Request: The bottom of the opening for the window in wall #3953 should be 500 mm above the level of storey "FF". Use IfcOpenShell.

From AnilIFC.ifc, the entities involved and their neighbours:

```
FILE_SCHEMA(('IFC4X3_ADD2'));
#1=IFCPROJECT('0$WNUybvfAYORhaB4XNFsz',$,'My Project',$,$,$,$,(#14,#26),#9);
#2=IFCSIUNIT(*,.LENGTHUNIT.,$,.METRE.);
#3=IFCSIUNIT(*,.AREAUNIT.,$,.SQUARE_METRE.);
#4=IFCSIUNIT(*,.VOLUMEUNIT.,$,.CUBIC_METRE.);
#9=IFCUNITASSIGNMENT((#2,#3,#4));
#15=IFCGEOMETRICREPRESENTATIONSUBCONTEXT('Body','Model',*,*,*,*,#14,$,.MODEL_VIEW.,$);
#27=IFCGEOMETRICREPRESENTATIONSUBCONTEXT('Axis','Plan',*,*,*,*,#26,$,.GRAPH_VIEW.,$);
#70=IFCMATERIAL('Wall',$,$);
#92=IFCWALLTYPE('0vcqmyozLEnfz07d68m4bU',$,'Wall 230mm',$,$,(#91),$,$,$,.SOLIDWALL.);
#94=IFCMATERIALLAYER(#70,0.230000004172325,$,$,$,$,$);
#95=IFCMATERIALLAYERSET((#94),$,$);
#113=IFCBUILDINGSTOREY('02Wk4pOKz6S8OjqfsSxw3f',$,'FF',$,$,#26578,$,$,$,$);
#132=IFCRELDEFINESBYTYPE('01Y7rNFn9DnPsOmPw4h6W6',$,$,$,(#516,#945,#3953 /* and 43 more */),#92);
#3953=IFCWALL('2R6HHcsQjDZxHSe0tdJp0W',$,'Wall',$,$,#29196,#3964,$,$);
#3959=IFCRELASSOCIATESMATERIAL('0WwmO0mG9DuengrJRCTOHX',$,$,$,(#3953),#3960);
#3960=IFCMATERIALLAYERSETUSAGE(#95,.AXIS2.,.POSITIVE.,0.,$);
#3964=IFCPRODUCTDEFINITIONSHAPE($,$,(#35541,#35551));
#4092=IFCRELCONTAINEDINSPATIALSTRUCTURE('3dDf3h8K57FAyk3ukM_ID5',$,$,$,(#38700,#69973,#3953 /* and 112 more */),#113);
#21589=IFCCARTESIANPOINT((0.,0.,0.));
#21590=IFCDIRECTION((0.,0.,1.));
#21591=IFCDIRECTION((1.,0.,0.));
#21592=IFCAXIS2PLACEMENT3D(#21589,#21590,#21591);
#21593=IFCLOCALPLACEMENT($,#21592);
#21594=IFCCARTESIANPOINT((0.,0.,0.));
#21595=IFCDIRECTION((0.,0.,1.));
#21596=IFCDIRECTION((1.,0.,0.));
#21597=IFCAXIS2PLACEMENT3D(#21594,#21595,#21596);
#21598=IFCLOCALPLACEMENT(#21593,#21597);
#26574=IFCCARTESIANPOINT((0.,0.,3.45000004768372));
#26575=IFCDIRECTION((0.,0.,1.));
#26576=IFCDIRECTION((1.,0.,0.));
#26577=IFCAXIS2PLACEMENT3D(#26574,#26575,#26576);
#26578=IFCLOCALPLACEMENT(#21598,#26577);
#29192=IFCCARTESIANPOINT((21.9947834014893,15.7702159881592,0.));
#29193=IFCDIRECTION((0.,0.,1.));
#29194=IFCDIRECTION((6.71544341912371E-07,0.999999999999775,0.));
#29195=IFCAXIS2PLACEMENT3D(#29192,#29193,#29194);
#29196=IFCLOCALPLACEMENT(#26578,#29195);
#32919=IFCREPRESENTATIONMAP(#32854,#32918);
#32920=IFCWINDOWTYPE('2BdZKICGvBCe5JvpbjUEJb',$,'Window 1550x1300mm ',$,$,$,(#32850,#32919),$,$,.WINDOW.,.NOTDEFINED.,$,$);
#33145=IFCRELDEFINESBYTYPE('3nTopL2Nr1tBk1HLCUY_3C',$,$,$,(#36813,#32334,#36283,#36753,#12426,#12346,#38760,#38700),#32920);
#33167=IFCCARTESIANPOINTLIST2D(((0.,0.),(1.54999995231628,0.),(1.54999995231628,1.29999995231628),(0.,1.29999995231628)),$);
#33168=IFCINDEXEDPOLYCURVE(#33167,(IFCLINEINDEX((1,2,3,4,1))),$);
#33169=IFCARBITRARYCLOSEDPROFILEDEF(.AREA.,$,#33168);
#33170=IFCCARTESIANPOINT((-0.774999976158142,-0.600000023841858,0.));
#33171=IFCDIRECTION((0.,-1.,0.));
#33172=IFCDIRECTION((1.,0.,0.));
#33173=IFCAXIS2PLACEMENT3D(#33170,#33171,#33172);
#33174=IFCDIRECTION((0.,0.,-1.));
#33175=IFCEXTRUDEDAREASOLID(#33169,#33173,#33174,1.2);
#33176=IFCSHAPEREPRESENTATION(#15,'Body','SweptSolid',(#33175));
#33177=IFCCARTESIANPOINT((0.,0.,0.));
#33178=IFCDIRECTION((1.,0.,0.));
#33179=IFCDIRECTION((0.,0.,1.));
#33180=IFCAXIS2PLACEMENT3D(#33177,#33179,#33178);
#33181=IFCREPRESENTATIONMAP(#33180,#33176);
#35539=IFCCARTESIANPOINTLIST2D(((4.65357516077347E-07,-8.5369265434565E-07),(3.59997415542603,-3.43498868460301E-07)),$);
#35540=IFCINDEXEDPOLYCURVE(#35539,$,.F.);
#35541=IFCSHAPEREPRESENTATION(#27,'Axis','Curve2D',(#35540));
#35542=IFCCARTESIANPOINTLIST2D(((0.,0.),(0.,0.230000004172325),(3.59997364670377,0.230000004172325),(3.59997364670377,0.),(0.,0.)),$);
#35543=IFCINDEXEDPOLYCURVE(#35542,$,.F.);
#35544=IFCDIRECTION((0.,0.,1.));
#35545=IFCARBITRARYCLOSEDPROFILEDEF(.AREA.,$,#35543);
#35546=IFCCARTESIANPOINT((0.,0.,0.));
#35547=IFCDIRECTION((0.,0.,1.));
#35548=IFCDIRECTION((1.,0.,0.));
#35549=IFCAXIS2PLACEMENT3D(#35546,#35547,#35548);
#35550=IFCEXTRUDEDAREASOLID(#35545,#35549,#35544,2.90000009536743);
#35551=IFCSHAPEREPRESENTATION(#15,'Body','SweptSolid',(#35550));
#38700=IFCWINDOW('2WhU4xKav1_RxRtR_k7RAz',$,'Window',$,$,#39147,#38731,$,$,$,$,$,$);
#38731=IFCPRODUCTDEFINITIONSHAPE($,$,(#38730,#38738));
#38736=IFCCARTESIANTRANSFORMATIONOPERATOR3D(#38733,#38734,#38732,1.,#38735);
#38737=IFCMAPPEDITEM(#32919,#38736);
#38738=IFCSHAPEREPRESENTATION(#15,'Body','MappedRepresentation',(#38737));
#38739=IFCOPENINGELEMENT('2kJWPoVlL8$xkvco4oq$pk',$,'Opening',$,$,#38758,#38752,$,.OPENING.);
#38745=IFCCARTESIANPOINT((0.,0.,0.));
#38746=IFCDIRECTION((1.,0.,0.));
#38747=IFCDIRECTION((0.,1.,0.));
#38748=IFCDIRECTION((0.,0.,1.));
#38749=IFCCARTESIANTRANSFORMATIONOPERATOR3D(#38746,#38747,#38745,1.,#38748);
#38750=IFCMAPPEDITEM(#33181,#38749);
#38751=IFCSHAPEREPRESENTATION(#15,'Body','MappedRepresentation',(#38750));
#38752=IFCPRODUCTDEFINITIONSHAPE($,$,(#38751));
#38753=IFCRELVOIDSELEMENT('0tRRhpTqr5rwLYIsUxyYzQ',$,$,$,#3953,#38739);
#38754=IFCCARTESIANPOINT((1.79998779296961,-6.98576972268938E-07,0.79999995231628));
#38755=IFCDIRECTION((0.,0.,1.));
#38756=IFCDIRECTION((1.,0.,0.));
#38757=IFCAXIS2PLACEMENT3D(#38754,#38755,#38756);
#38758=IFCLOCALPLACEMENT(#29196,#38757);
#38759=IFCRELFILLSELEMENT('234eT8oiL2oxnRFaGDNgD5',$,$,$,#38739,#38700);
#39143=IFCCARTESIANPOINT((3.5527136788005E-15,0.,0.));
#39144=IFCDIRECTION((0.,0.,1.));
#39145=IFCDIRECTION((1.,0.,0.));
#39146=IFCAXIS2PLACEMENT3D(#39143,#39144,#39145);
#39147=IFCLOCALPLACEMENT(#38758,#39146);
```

```python
import numpy as np
import ifcopenshell
import ifcopenshell.api.geometry
import ifcopenshell.geom
import ifcopenshell.util.element
import ifcopenshell.util.placement
import ifcopenshell.util.shape
import ifcopenshell.util.unit

model = ifcopenshell.open("AnilIFC.ifc")
unit_scale = ifcopenshell.util.unit.calculate_unit_scale(model)

window = model.by_id(38700)
opening = window.FillsVoids[0].RelatingOpeningElement
storey = ifcopenshell.util.element.get_container(window, ifc_class="IfcBuildingStorey")
level = ifcopenshell.util.placement.get_local_placement(storey.ObjectPlacement)[2, 3]

# The opening's origin need not be at the sill, so measure its lowest point.
shape = ifcopenshell.geom.create_shape(ifcopenshell.geom.settings(), opening)
bottom = ifcopenshell.util.shape.get_shape_bottom_elevation(shape, shape.geometry) / unit_scale
dz = level + 0.5 / unit_scale - bottom

shift = np.array([0.0, 0.0, dz])
# The window is placed relative to its opening, so it follows when the opening moves.
matrix = ifcopenshell.util.placement.get_local_placement(opening.ObjectPlacement)
matrix[:3, 3] += shift
ifcopenshell.api.geometry.edit_object_placement(
    model, product=opening, matrix=matrix, is_si=False, should_transform_children=True
)

print(f"moved by {dz * unit_scale:+.3f} m")

model.write("AnilIFC_edited.ifc")
```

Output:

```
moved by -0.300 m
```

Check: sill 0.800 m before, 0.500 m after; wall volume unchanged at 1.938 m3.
